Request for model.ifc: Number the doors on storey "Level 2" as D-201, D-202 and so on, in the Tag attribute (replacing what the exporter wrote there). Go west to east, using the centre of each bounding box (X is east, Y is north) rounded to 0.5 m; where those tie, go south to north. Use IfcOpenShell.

First a look at what the model holds.

```python
import ifcopenshell
import ifcopenshell.util.element
import ifcopenshell.util.placement

model = ifcopenshell.open("model.ifc")
print(model.schema)
storey = next(s for s in model.by_type("IfcBuildingStorey") if s.Name == "Level 2")
doors = [e for e in ifcopenshell.util.element.get_decomposition(storey) if e.is_a("IfcDoor")]
for e in sorted(doors, key=lambda e: e.id()):
    origin = ifcopenshell.util.placement.get_local_placement(e.ObjectPlacement)[:3, 3]
    print(e.id(), e.Tag, e.Name, origin.round(2) + 0.0, sep=" | ")
```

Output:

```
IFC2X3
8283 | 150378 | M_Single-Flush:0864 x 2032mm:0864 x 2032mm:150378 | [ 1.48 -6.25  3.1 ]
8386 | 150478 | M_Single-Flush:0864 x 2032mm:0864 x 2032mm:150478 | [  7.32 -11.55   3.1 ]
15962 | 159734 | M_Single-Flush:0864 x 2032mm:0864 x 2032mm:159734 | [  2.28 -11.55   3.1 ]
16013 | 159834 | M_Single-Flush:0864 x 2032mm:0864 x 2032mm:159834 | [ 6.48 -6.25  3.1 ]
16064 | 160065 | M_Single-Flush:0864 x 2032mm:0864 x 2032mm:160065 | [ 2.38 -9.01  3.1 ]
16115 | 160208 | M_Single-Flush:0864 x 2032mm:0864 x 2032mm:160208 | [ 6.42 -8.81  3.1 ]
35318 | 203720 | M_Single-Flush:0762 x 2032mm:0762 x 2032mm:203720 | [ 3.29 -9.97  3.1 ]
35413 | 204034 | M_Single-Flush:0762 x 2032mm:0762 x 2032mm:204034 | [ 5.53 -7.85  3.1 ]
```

```python
import ifcopenshell
import ifcopenshell.geom
import ifcopenshell.util.element
import ifcopenshell.util.shape

model = ifcopenshell.open("model.ifc")
settings = ifcopenshell.geom.settings()
settings.set("use-world-coords", True)


def centre(element):
    shape = ifcopenshell.geom.create_shape(settings, element)
    return ifcopenshell.util.shape.get_bbox_centroid(shape.geometry)


storey = next(s for s in model.by_type("IfcBuildingStorey") if s.Name == "Level 2")
doors = [e for e in ifcopenshell.util.element.get_decomposition(storey) if e.is_a("IfcDoor")]

# Insertion points can sit at a corner or the storey origin, so sort by the geometry (in metres).
centres = {e: centre(e) for e in doors}
doors.sort(key=lambda e: (round(centres[e][0] / 0.5), centres[e][1]))

for i, e in enumerate(doors, start=1):
    number = f"D-2{i:02d}"
    e.Tag = number
    print(e.id(), number)

model.write("model-out.ifc")
```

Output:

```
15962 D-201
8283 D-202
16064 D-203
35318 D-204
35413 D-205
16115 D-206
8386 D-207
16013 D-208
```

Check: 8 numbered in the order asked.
